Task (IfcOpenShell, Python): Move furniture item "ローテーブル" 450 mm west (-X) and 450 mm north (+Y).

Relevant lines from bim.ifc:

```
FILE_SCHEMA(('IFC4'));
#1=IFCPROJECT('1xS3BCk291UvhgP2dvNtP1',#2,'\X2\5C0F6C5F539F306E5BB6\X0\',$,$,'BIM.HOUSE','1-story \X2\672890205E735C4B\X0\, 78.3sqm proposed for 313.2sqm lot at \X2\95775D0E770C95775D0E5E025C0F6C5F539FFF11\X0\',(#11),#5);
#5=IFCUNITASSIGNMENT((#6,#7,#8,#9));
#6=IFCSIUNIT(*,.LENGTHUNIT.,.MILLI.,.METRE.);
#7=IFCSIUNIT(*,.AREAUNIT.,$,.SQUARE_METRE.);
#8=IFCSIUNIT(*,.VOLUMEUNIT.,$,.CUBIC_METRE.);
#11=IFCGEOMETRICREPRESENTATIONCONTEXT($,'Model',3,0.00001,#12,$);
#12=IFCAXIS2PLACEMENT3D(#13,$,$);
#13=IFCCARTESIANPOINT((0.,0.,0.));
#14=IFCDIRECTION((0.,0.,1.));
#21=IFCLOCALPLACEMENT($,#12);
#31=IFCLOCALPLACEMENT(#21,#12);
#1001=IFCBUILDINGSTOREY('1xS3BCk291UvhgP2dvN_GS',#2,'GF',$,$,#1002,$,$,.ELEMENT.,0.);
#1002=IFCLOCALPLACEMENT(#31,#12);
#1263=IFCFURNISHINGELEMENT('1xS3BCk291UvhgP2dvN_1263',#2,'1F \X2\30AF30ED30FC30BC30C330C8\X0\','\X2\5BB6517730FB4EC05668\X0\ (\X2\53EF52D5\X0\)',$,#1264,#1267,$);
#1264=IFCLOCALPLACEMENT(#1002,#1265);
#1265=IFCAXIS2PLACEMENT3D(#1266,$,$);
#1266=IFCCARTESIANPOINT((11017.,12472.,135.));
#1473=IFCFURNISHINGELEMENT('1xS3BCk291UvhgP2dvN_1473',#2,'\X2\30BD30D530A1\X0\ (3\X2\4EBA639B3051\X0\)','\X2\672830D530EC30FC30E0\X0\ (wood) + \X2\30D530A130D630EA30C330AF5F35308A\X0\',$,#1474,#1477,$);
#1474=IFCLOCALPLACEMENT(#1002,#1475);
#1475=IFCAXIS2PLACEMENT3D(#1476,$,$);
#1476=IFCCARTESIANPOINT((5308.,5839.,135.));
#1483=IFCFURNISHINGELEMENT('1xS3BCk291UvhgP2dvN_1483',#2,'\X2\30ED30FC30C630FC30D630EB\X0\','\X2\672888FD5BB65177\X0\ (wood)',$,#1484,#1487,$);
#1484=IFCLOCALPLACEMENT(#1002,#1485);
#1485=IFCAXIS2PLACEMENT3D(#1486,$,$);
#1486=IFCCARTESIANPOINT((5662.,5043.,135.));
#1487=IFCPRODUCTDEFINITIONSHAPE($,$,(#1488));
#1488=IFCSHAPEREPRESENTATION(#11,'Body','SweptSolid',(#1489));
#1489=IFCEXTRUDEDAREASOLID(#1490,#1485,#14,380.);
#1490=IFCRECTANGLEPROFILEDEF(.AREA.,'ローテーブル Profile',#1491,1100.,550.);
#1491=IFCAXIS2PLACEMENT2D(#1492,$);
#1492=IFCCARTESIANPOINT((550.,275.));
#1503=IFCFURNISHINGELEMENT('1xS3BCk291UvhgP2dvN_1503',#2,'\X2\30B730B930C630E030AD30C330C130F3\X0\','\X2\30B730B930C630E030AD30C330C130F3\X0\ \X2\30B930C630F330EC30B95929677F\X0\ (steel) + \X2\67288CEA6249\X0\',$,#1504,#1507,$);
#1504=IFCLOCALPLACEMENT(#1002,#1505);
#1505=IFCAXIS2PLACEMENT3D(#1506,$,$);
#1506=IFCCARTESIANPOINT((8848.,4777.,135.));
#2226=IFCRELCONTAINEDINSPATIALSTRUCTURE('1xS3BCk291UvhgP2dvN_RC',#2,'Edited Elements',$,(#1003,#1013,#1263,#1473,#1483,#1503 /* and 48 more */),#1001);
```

```python
import ifcopenshell
import ifcopenshell.api.geometry
import ifcopenshell.util.placement

model = ifcopenshell.open("bim.ifc")

item = model.by_id(1483)
matrix = ifcopenshell.util.placement.get_local_placement(item.ObjectPlacement)
matrix[0, 3] -= 450.0
matrix[1, 3] += 450.0
ifcopenshell.api.geometry.edit_object_placement(model, product=item, matrix=matrix, is_si=False)

print(ifcopenshell.util.placement.get_local_placement(item.ObjectPlacement).round(3) + 0.0)

model.write("bim_v2.ifc")
```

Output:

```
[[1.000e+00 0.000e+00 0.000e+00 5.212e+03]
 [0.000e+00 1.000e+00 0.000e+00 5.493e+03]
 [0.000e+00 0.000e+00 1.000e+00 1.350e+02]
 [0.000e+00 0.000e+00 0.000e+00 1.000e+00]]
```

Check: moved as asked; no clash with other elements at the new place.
